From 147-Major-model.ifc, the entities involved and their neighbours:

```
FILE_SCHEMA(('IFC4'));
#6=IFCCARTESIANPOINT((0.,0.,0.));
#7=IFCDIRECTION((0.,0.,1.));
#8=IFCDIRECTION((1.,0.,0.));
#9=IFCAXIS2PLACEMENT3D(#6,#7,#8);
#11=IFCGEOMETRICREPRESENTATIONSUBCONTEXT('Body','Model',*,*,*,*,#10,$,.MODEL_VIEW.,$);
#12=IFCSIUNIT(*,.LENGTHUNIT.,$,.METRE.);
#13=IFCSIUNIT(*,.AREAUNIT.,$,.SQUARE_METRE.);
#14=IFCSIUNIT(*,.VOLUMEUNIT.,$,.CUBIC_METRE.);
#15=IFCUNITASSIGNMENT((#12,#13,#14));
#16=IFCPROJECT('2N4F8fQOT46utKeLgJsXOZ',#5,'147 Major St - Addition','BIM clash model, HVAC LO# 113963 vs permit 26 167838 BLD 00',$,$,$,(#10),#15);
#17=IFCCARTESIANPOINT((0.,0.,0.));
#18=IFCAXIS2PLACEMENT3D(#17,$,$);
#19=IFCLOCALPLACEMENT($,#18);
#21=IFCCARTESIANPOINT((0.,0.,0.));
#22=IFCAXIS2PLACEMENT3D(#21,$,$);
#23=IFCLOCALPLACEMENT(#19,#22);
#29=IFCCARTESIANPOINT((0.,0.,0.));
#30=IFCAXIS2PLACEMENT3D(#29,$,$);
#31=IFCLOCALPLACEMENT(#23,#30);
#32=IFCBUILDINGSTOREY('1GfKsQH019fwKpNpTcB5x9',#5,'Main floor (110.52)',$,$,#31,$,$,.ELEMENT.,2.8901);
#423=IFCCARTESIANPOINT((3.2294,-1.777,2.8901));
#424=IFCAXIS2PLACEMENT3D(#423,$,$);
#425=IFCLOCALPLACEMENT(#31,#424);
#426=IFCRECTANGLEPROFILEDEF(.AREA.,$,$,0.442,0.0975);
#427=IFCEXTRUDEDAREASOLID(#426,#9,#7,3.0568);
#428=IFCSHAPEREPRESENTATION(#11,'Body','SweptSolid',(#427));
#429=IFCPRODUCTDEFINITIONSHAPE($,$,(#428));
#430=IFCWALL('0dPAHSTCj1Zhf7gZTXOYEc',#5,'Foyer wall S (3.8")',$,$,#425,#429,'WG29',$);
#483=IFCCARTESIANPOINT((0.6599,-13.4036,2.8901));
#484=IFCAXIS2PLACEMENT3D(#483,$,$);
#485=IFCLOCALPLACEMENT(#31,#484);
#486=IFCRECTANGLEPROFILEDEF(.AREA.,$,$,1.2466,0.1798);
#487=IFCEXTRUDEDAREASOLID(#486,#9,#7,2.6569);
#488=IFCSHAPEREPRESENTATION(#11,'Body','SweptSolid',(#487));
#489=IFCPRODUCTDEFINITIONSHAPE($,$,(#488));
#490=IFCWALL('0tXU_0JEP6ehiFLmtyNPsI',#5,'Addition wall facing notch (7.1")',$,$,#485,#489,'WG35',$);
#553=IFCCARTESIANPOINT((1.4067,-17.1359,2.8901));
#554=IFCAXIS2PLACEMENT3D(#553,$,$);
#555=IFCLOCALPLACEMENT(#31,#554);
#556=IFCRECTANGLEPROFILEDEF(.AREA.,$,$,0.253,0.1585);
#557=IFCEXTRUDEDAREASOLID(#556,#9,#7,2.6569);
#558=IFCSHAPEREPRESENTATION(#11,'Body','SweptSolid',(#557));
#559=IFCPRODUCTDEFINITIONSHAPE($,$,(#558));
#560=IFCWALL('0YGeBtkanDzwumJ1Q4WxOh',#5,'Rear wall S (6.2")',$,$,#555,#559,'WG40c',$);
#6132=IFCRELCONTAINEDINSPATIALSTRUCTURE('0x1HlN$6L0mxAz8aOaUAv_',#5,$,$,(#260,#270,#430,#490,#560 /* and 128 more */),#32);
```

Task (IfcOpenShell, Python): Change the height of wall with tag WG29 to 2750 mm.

```python
import ifcopenshell
import ifcopenshell.geom
import ifcopenshell.util.representation
import ifcopenshell.util.shape
import ifcopenshell.util.unit

model = ifcopenshell.open("147-Major-model.ifc")
unit_scale = ifcopenshell.util.unit.calculate_unit_scale(model)
settings = ifcopenshell.geom.settings()


def volume(element):
    """Net volume in cubic metres, openings subtracted."""
    shape = ifcopenshell.geom.create_shape(settings, element)
    return ifcopenshell.util.shape.get_volume(shape.geometry)


wall = model.by_guid("0dPAHSTCj1Zhf7gZTXOYEc")
before = volume(wall)

body = ifcopenshell.util.representation.get_representation(wall, "Model", "Body")
solid = body.Items[0]
old_height = solid.Depth
solid.Depth = 2.75 / unit_scale
after = volume(wall)

print(f"height {old_height:g} -> {solid.Depth:g}, volume {before:.3f} -> {after:.3f} m3")

model.write("147-Major-model-out.ifc")
```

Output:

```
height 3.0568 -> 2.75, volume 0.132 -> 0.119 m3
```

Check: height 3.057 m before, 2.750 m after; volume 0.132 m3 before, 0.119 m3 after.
